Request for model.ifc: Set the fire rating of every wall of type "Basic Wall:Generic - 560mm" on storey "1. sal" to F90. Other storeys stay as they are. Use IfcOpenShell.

First a look at what the model holds.

```python
import ifcopenshell
import ifcopenshell.util.element

model = ifcopenshell.open("model.ifc")
print(model.schema)
storey = next(s for s in model.by_type("IfcBuildingStorey") if s.Name == "1. sal")
walls = [e for e in ifcopenshell.util.element.get_decomposition(storey) if e.is_a("IfcWall")]
seen = {}
for e in walls:
    element_type = ifcopenshell.util.element.get_type(e)
    key = (element_type.Name if element_type != e and element_type else None, ifcopenshell.util.element.get_pset(e, "Pset_WallCommon", "FireRating"))
    seen[key] = seen.get(key, 0) + 1
for (name, value), count in sorted(seen.items(), key=str):
    print(count, "x", name, "|", value)
```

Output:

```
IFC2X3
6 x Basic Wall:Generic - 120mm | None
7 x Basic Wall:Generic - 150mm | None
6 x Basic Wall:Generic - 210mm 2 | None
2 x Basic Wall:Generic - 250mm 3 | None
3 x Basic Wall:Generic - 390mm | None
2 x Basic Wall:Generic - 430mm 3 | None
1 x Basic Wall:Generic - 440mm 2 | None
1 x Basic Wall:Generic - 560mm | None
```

```python
import ifcopenshell
import ifcopenshell.api.pset
import ifcopenshell.util.element

model = ifcopenshell.open("model.ifc")

storey = next(s for s in model.by_type("IfcBuildingStorey") if s.Name == "1. sal")
walls = [e for e in ifcopenshell.util.element.get_decomposition(storey) if e.is_a("IfcWall")]

count = 0
for e in walls:
    element_type = ifcopenshell.util.element.get_type(e)
    if element_type in (None, e) or element_type.Name != "Basic Wall:Generic - 560mm":
        continue
    # add_pset returns the element's existing set when there is one.
    pset = ifcopenshell.api.pset.add_pset(model, product=e, name="Pset_WallCommon")
    ifcopenshell.api.pset.edit_pset(model, pset=pset, properties={"FireRating": "F90"})
    count += 1

print(count, "walls updated")

model.write("model_rev.ifc")
```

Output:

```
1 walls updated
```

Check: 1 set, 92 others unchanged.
